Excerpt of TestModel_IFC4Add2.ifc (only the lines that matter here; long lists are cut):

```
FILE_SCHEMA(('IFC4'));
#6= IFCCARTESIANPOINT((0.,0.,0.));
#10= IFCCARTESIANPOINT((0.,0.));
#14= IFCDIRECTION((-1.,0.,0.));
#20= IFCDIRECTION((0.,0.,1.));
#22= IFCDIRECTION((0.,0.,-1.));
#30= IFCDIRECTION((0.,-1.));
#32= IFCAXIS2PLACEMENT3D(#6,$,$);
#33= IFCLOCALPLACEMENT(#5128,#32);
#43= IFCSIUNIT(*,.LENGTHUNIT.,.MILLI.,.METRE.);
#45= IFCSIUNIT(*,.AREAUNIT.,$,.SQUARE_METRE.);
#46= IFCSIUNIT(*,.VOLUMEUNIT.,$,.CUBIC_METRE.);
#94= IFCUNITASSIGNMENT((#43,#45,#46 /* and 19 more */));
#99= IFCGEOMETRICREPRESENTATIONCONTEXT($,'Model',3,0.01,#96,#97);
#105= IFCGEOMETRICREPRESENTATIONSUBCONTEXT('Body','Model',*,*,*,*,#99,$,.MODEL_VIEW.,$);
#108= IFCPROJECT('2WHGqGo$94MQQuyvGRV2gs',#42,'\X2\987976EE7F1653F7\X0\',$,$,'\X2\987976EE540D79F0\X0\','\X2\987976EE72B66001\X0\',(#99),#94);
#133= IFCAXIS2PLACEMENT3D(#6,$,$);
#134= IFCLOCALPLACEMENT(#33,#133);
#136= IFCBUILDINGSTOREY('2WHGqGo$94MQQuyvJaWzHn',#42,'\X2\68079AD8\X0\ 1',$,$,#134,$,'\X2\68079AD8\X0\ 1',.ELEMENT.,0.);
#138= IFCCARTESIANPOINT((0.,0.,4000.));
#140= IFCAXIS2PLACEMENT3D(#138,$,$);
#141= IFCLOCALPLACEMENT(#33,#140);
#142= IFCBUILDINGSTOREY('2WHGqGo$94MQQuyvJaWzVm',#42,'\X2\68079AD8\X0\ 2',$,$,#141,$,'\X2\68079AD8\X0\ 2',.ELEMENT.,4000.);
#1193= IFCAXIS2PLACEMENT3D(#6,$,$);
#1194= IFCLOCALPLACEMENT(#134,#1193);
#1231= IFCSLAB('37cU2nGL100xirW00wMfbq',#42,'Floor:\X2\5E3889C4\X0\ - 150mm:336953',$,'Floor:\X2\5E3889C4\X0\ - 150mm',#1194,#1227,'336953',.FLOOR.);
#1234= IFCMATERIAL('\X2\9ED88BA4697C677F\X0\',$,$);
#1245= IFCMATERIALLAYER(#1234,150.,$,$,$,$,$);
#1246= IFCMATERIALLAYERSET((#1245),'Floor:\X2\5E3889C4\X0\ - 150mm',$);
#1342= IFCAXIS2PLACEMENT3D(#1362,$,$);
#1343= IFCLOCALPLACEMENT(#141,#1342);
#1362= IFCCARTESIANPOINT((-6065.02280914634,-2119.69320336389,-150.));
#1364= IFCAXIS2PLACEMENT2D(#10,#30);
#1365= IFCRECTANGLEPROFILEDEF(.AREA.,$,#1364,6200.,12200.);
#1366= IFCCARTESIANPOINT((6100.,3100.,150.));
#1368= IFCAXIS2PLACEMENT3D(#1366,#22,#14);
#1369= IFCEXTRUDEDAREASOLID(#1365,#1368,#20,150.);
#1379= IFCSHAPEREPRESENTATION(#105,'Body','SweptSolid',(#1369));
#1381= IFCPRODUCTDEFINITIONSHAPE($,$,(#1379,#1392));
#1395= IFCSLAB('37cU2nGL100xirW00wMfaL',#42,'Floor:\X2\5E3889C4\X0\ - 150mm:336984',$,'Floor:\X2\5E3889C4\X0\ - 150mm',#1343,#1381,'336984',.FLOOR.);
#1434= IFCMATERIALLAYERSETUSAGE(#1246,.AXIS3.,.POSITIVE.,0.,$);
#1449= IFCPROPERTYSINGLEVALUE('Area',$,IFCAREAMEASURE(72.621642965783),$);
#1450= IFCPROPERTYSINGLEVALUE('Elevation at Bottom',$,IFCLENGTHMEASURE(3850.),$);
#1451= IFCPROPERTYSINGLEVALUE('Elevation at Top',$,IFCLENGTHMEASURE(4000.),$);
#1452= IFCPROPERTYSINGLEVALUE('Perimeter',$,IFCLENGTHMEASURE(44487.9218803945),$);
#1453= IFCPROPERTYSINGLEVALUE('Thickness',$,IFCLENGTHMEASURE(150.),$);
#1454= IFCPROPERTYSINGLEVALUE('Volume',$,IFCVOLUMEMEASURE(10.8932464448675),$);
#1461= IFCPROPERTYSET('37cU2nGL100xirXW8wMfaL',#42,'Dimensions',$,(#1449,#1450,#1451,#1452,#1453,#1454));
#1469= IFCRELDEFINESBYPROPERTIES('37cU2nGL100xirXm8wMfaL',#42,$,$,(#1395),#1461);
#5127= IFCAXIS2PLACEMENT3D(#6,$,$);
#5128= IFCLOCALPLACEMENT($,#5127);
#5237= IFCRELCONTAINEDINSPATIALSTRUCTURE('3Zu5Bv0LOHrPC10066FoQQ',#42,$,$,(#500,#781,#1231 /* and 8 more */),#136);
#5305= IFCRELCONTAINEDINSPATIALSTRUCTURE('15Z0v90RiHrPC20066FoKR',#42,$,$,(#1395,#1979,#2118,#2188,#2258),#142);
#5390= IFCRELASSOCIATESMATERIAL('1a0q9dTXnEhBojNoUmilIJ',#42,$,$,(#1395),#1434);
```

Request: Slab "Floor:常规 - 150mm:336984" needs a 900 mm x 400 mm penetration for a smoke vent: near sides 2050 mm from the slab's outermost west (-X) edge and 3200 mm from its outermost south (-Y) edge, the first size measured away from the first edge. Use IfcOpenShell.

```python
import numpy as np
import ifcopenshell
import ifcopenshell.api.feature
import ifcopenshell.api.geometry
import ifcopenshell.api.pset
import ifcopenshell.api.root
import ifcopenshell.geom
import ifcopenshell.util.element
import ifcopenshell.util.placement
import ifcopenshell.util.representation
import ifcopenshell.util.shape
import ifcopenshell.util.unit

model = ifcopenshell.open("TestModel_IFC4Add2.ifc")
unit_scale = ifcopenshell.util.unit.calculate_unit_scale(model)
area_scale = ifcopenshell.util.unit.calculate_unit_scale(model, "AREAUNIT")
volume_scale = ifcopenshell.util.unit.calculate_unit_scale(model, "VOLUMEUNIT")
settings = ifcopenshell.geom.settings()


def volume(element):
    """Net volume in cubic metres, openings subtracted."""
    shape = ifcopenshell.geom.create_shape(settings, element)
    return ifcopenshell.util.shape.get_volume(shape.geometry)


slab = model.by_guid("37cU2nGL100xirW00wMfaL")
before = volume(slab)

# Extent in the slab's own axes, in metres. The edges named are its -X and -Y sides.
slab_shape = ifcopenshell.geom.create_shape(settings, slab)
vertices = ifcopenshell.util.shape.get_vertices(slab_shape.geometry)
x_min, y_min, bottom = vertices.min(axis=0)
top = vertices[:, 2].max()

opening = ifcopenshell.api.root.create_entity(model, ifc_class="IfcOpeningElement", name="Smoke vent opening", predefined_type="OPENING")
context = ifcopenshell.util.representation.get_context(model, "Model", "Body", "MODEL_VIEW")
width, depth = 0.9, 0.4
outline = [(0.0, 0.0), (width, 0.0), (width, depth), (0.0, depth), (0.0, 0.0)]
# Overshoot both faces by 50 mm so the cut is clean.
shape = ifcopenshell.api.geometry.add_slab_representation(
    model, context=context, depth=top - bottom + 0.1, polyline=outline
)
ifcopenshell.api.geometry.assign_representation(model, product=opening, representation=shape)

matrix = ifcopenshell.util.placement.get_local_placement(slab.ObjectPlacement)
matrix[:, 3] = matrix @ np.append(np.array([x_min + 2.05, y_min + 3.2, bottom - 0.05]) / unit_scale, 1.0)
ifcopenshell.api.geometry.edit_object_placement(model, product=opening, matrix=matrix, is_si=False)
ifcopenshell.api.feature.add_feature(model, feature=opening, element=slab)

after = volume(slab)

# Update the slab's stored quantities.
pset = model.by_id(ifcopenshell.util.element.get_pset(slab, "Dimensions", should_inherit=False)["id"])
ifcopenshell.api.pset.edit_pset(model, pset=pset, properties={
    "Area": model.create_entity("IfcAreaMeasure", after / (top - bottom) / area_scale),
    "Volume": model.create_entity("IfcVolumeMeasure", after / volume_scale),
})

print(f"slab volume {before:.3f} -> {after:.3f} m3")

model.write("TestModel_IFC4Add2-out.ifc")
```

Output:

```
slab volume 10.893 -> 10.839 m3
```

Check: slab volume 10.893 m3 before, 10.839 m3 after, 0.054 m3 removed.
